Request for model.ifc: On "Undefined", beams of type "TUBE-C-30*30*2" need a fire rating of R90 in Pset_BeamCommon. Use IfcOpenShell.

First a look at what the model holds.

```python
import ifcopenshell
import ifcopenshell.util.element

model = ifcopenshell.open("model.ifc")
print(model.schema)
storey = next(s for s in model.by_type("IfcBuildingStorey") if s.Name == "Undefined")
beams = [e for e in ifcopenshell.util.element.get_decomposition(storey) if e.is_a("IfcBeam")]
seen = {}
for e in beams:
    element_type = ifcopenshell.util.element.get_type(e)
    key = (element_type.Name if element_type != e and element_type else None, ifcopenshell.util.element.get_pset(e, "Pset_BeamCommon", "FireRating"))
    seen[key] = seen.get(key, 0) + 1
for (name, value), count in sorted(seen.items(), key=str):
    print(count, "x", name, "|", value)
```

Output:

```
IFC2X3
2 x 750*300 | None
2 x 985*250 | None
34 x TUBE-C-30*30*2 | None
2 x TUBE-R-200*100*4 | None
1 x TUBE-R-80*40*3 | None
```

```python
import ifcopenshell
import ifcopenshell.api.pset
import ifcopenshell.util.element

model = ifcopenshell.open("model.ifc")

storey = next(s for s in model.by_type("IfcBuildingStorey") if s.Name == "Undefined")
beams = [e for e in ifcopenshell.util.element.get_decomposition(storey) if e.is_a("IfcBeam")]

count = 0
for e in beams:
    element_type = ifcopenshell.util.element.get_type(e)
    if element_type in (None, e) or element_type.Name != "TUBE-C-30*30*2":
        continue
    # add_pset returns the element's existing set when there is one.
    pset = ifcopenshell.api.pset.add_pset(model, product=e, name="Pset_BeamCommon")
    ifcopenshell.api.pset.edit_pset(model, pset=pset, properties={"FireRating": "R90"})
    count += 1

print(count, "beams updated")

model.write("model_edited.ifc")
```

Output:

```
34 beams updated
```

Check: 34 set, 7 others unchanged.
